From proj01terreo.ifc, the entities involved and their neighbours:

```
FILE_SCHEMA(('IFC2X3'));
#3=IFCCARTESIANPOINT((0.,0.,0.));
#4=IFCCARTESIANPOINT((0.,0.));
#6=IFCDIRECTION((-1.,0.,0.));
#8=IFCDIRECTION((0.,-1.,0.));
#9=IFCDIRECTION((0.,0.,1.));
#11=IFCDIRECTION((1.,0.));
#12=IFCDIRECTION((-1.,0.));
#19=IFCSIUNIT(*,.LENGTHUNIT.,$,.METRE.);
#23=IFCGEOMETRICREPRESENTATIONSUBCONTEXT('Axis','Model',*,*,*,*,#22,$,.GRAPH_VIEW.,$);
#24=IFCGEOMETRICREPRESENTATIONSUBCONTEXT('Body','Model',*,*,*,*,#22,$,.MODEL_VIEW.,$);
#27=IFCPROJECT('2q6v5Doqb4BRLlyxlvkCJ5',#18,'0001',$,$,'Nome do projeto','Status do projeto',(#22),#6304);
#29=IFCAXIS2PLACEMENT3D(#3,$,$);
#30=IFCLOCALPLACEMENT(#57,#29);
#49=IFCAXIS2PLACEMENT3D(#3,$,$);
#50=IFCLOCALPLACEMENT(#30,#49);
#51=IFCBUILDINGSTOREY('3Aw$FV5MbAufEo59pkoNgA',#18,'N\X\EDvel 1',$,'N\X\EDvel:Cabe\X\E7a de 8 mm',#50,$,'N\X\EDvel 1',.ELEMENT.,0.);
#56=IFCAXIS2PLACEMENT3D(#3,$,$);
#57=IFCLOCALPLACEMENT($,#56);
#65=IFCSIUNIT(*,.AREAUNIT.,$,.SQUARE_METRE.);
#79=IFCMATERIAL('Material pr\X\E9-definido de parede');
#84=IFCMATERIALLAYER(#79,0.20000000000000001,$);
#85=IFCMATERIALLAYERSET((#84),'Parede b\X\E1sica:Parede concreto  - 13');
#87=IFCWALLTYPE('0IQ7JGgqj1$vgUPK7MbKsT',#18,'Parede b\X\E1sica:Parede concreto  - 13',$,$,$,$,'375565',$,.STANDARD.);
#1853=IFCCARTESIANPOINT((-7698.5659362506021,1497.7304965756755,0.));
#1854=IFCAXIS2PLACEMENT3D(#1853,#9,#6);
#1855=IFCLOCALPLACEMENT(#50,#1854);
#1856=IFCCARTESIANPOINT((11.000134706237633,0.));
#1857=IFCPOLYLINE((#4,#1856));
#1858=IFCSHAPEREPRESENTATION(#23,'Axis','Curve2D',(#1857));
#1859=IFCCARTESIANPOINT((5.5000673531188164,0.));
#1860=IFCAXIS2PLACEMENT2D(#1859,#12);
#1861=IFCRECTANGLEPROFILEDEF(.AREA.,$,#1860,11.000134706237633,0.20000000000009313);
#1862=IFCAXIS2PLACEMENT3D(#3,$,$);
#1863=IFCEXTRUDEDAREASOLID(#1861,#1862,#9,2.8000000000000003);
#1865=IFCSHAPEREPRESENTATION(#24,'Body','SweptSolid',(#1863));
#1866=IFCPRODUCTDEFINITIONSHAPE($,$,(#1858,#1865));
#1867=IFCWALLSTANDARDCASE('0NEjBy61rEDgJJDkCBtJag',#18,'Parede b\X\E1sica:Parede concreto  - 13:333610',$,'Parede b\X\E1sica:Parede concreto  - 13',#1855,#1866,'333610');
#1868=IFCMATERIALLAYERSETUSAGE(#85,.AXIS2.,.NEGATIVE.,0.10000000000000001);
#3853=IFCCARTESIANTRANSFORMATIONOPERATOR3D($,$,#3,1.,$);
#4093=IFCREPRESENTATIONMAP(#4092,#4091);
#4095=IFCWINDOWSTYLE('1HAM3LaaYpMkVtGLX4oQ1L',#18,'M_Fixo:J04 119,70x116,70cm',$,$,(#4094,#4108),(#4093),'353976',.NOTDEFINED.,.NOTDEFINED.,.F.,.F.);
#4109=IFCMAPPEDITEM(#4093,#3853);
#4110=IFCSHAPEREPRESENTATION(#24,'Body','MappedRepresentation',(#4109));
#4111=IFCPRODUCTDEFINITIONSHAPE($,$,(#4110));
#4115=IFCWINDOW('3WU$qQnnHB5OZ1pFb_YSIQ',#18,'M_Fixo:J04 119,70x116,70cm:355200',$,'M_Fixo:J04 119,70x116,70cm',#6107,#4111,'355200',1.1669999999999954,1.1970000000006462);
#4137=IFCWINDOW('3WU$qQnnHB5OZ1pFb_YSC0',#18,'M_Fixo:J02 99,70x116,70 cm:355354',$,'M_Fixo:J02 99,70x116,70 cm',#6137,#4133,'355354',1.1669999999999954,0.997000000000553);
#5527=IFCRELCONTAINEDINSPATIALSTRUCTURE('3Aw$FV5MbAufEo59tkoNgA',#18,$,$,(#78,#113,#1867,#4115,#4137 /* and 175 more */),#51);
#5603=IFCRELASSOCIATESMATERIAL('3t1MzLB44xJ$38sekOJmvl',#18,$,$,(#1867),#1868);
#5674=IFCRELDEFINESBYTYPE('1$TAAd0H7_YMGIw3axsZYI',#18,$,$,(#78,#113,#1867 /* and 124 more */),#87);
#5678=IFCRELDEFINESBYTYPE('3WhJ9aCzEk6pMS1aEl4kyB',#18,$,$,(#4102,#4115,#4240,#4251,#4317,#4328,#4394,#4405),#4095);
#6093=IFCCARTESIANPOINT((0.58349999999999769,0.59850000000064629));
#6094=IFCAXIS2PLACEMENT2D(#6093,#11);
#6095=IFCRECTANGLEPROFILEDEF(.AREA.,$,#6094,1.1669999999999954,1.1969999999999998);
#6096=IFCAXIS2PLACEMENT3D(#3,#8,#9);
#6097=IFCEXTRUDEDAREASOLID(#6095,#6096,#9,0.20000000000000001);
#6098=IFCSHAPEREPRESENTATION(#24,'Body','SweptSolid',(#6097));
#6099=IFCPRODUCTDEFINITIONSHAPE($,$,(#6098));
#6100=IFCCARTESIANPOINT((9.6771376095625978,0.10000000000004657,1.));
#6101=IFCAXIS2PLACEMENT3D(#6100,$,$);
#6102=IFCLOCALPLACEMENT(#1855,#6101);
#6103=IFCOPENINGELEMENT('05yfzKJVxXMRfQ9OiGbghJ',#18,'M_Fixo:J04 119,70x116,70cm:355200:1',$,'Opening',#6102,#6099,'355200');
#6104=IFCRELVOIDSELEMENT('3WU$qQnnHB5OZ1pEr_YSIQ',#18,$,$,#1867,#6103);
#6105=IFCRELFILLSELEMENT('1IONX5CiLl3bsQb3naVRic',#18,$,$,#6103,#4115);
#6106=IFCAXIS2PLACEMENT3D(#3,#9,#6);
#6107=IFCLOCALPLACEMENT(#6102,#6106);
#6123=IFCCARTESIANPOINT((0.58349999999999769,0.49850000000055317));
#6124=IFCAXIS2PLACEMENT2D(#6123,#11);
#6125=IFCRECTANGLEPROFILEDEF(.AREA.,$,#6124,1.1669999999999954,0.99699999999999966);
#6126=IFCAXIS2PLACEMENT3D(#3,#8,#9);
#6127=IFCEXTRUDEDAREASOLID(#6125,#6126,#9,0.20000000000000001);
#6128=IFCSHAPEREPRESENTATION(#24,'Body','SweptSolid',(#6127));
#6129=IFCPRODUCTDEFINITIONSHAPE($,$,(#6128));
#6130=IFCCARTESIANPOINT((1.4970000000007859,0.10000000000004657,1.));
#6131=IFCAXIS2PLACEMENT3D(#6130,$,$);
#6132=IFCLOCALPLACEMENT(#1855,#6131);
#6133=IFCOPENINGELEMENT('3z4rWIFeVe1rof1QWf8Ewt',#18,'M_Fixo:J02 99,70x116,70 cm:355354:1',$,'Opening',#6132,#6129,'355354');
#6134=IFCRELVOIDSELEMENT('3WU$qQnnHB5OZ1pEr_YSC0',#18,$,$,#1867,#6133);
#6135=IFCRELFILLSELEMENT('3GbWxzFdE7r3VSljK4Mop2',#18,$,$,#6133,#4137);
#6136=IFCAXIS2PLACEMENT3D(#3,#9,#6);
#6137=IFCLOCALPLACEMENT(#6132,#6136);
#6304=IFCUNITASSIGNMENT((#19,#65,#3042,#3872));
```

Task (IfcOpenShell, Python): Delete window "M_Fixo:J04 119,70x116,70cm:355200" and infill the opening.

```python
import ifcopenshell
import ifcopenshell.api.feature
import ifcopenshell.api.root
import ifcopenshell.geom
import ifcopenshell.util.shape

model = ifcopenshell.open("proj01terreo.ifc")
settings = ifcopenshell.geom.settings()


def volume(element):
    """Net volume in cubic metres, openings subtracted."""
    shape = ifcopenshell.geom.create_shape(settings, element)
    return ifcopenshell.util.shape.get_volume(shape.geometry)


window = model.by_guid("3WU$qQnnHB5OZ1pFb_YSIQ")
opening = window.FillsVoids[0].RelatingOpeningElement
wall = opening.VoidsElements[0].RelatingBuildingElement
before = volume(wall)

ifcopenshell.api.root.remove_product(model, product=window)
ifcopenshell.api.feature.remove_feature(model, feature=opening)

after = volume(wall)

print(f"wall volume {before:.3f} -> {after:.3f} m3")

model.write("proj01terreo_rev.ifc")
```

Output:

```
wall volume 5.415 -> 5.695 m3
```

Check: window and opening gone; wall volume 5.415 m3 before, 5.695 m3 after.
